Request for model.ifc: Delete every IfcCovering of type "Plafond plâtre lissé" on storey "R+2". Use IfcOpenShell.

First a look at what the model holds.

```python
import ifcopenshell
import ifcopenshell.util.element

model = ifcopenshell.open("model.ifc")
print(model.schema)
storey = next(s for s in model.by_type("IfcBuildingStorey") if s.Name == "R+2")
coverings = [e for e in ifcopenshell.util.element.get_decomposition(storey) if e.is_a("IfcCovering")]
seen = {}
for e in coverings:
    element_type = ifcopenshell.util.element.get_type(e)
    name = element_type.Name if element_type not in (None, e) else None
    seen[name] = seen.get(name, 0) + 1
for name, count in sorted(seen.items(), key=str):
    print(count, "x", name)
```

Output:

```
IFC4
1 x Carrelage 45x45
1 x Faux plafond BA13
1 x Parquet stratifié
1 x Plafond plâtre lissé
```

```python
import ifcopenshell
import ifcopenshell.api.root
import ifcopenshell.util.element

model = ifcopenshell.open("model.ifc")

storey = next(s for s in model.by_type("IfcBuildingStorey") if s.Name == "R+2")
coverings = [e for e in ifcopenshell.util.element.get_decomposition(storey) if e.is_a("IfcCovering")]
targets = [e for e in coverings if (t := ifcopenshell.util.element.get_type(e)) not in (None, e) and t.Name == "Plafond plâtre lissé"]

for e in targets:
    ifcopenshell.api.root.remove_product(model, product=e)
print(len(targets), "removed")

model.write("model_updated.ifc")
```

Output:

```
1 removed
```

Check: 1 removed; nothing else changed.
